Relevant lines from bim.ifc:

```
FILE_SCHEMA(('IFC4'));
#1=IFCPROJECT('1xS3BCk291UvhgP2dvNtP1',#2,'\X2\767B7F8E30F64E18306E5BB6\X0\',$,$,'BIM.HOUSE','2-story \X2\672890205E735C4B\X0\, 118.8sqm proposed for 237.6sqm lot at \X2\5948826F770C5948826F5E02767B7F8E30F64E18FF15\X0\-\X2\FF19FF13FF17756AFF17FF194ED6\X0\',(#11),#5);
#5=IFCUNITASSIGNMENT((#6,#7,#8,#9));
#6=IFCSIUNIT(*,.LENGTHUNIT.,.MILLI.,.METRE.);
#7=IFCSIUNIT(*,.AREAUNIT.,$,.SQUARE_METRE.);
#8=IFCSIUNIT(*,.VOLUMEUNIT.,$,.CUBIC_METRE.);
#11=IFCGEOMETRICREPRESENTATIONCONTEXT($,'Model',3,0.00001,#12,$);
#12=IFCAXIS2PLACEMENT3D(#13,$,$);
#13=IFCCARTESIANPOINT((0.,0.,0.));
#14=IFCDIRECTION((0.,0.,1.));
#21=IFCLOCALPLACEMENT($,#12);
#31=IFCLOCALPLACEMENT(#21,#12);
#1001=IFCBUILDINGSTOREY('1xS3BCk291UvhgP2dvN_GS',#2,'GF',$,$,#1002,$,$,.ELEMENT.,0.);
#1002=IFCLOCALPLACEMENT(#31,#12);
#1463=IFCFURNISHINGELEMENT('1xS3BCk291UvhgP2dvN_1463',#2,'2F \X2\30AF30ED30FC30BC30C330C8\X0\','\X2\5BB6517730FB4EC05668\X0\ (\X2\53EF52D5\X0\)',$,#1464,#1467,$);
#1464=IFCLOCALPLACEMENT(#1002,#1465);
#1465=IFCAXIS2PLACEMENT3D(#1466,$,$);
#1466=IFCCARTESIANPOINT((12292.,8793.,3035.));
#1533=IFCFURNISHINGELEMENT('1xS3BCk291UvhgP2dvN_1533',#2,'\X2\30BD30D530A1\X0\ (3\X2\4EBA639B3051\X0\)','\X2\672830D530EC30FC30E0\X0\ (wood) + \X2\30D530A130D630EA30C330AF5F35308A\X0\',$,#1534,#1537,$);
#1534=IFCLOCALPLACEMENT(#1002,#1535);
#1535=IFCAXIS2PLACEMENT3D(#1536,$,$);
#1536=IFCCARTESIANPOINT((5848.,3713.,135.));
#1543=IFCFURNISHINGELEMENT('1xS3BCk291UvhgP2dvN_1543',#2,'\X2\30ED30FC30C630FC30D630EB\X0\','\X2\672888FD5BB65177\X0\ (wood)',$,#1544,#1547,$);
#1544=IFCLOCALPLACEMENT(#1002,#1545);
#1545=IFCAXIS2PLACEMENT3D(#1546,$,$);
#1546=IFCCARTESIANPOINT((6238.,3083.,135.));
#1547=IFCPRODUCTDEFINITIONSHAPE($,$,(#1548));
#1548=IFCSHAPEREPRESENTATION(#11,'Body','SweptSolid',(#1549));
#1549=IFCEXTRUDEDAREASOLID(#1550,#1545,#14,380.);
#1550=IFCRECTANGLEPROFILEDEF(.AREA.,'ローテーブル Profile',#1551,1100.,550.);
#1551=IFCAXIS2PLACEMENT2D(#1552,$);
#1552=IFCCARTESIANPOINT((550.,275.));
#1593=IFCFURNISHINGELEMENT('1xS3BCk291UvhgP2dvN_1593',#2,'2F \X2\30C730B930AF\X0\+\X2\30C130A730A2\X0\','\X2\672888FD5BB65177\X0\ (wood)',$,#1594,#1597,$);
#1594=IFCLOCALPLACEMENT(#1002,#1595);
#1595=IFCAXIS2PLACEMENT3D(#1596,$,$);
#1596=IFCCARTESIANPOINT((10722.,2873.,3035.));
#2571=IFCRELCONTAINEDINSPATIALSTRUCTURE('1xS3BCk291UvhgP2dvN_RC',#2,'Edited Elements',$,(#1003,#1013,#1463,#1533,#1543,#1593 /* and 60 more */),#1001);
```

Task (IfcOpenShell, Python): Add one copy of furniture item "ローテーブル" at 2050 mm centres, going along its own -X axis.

```python
import ifcopenshell
import ifcopenshell.api.geometry
import ifcopenshell.api.root
import ifcopenshell.util.element
import ifcopenshell.util.placement
import ifcopenshell.util.unit

model = ifcopenshell.open("bim.ifc")
unit_scale = ifcopenshell.util.unit.calculate_unit_scale(model)


def reuse_history(source, copy):
    """copy_class also copies each property set's owner history, people and application; keep the originals."""
    for rel in copy.IsDefinedBy:
        if rel.is_a("IfcRelDefinesByProperties") and (history := rel.RelatingPropertyDefinition.OwnerHistory):
            rel.RelatingPropertyDefinition.OwnerHistory = source.OwnerHistory
            ifcopenshell.util.element.remove_deep2(model, history)


source = model.by_guid("1xS3BCk291UvhgP2dvN_1543")
base = ifcopenshell.util.placement.get_local_placement(source.ObjectPlacement)
step = -base[:3, 0] * 2.05 / unit_scale

for i in range(1, 2):
    copy = ifcopenshell.api.root.copy_class(model, product=source)
    copy.Representation = ifcopenshell.util.element.copy_deep(
        model, source.Representation, exclude=["IfcGeometricRepresentationContext", "IfcRepresentationMap"]
    )
    reuse_history(source, copy)
    matrix = base.copy()
    matrix[:3, 3] += i * step
    print("added at", matrix[:3, 3].round(3) + 0.0)
    ifcopenshell.api.geometry.edit_object_placement(model, product=copy, matrix=matrix, is_si=False)

model.write("bim_v2.ifc")
```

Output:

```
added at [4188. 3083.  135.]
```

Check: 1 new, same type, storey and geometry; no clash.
